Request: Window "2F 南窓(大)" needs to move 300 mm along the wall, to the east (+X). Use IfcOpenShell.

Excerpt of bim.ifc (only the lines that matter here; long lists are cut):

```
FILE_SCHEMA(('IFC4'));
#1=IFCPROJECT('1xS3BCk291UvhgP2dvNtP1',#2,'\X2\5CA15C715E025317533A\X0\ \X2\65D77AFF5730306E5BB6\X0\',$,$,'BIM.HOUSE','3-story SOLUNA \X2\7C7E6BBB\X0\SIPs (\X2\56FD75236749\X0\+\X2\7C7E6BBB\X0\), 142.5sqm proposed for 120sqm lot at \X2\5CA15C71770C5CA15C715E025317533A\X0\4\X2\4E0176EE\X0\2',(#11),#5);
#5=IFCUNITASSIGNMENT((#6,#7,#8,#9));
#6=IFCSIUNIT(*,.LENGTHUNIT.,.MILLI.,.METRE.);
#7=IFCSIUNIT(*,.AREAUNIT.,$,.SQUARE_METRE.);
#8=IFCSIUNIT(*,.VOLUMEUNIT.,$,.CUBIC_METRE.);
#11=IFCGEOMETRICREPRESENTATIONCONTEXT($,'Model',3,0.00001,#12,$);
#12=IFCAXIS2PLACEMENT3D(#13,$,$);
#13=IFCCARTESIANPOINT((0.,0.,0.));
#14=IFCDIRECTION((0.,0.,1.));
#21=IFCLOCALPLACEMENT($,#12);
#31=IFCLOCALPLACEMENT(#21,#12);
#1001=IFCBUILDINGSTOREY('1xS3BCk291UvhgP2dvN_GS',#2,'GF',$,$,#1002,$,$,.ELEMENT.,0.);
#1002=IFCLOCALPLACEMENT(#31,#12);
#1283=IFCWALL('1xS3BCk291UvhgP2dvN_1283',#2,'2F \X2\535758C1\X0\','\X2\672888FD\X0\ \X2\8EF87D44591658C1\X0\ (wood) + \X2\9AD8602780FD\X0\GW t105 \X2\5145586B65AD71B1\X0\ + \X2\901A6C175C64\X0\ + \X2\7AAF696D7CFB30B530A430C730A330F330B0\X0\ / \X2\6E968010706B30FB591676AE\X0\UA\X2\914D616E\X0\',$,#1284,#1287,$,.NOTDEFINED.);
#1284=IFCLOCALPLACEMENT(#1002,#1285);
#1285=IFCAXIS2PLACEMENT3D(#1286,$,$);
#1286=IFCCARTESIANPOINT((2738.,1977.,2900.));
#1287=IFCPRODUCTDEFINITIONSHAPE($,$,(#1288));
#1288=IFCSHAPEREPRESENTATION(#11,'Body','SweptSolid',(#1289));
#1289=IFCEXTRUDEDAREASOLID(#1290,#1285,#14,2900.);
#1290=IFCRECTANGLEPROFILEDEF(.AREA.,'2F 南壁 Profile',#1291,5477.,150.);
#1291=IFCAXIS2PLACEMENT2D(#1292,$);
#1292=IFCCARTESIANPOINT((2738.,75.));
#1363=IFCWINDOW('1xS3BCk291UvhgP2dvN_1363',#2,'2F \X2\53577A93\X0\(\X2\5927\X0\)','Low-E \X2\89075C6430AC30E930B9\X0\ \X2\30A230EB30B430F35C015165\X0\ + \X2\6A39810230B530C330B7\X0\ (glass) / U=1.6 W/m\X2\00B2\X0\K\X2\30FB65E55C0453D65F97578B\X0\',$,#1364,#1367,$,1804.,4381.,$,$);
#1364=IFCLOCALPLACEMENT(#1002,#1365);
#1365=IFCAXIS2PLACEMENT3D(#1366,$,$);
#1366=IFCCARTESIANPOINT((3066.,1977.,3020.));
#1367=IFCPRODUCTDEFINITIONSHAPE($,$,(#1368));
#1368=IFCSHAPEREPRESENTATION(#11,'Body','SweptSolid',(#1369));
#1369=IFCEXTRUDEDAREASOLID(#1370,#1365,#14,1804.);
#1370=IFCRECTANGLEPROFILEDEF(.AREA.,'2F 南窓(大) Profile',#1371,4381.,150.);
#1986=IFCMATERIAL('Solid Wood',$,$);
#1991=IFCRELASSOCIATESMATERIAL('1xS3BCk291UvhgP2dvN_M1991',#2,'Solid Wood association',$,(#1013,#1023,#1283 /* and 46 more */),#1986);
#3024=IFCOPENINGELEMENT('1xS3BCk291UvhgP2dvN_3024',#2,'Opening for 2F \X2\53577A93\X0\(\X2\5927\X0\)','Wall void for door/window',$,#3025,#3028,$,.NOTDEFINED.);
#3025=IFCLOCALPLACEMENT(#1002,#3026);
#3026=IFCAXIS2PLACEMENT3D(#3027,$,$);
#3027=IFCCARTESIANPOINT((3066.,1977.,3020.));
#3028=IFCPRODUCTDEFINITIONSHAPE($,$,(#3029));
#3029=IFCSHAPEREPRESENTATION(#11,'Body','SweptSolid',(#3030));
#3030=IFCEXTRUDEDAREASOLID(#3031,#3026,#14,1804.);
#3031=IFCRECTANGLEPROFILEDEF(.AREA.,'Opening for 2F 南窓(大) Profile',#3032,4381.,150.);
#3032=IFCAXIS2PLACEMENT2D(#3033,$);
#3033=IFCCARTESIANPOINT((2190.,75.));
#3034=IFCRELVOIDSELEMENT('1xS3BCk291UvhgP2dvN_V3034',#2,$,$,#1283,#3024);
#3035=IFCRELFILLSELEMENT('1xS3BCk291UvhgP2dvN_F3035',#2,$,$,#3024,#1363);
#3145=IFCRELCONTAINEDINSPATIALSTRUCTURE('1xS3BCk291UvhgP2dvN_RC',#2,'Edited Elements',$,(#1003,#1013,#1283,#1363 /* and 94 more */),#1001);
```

```python
import ifcopenshell
import ifcopenshell.api.geometry
import ifcopenshell.util.placement

model = ifcopenshell.open("bim.ifc")

window = model.by_id(1363)
opening = window.FillsVoids[0].RelatingOpeningElement
wall = opening.VoidsElements[0].RelatingBuildingElement

wall_matrix = ifcopenshell.util.placement.get_local_placement(wall.ObjectPlacement)
shift = wall_matrix[:3, 0] * 300.0
before = ifcopenshell.util.placement.get_local_placement(window.ObjectPlacement)[:3, 3].copy()

# The window is not placed relative to its opening, so move both.
for product in (opening, window):
    matrix = ifcopenshell.util.placement.get_local_placement(product.ObjectPlacement)
    matrix[:3, 3] += shift
    ifcopenshell.api.geometry.edit_object_placement(model, product=product, matrix=matrix, is_si=False)

after = ifcopenshell.util.placement.get_local_placement(window.ObjectPlacement)[:3, 3]
print("window moved by", (after - before).round(3) + 0.0)

model.write("bim_v2.ifc")
```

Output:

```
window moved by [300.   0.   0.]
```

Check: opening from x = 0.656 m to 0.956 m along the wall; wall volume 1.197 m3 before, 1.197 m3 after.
